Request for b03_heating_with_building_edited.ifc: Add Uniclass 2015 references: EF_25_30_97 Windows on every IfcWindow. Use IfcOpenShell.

First a look at what the model holds.

```python
import ifcopenshell

model = ifcopenshell.open("b03_heating_with_building_edited.ifc")
print(model.schema)
print("classifications:", [c.Name for c in model.by_type("IfcClassification")])
for ifc_class in ("IfcDoor", "IfcRoof", "IfcStair", "IfcWall", "IfcWindow"):
    print(ifc_class, len(model.by_type(ifc_class)))
```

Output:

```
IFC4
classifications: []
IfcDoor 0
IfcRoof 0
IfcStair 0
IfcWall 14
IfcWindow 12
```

```python
import ifcopenshell
import ifcopenshell.api.classification

model = ifcopenshell.open("b03_heating_with_building_edited.ifc")

system = ifcopenshell.api.classification.add_classification(model, classification="Uniclass 2015")

codes = {
    "IfcWindow": ("EF_25_30_97", "Windows"),
}
for ifc_class, (code, name) in codes.items():
    products = model.by_type(ifc_class)
    ifcopenshell.api.classification.add_reference(
        model, products=products, classification=system, identification=code, name=name
    )
    print(code, len(products))

model.write("b03_heating_with_building_edited_v2.ifc")
```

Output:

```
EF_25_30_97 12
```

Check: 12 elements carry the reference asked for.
